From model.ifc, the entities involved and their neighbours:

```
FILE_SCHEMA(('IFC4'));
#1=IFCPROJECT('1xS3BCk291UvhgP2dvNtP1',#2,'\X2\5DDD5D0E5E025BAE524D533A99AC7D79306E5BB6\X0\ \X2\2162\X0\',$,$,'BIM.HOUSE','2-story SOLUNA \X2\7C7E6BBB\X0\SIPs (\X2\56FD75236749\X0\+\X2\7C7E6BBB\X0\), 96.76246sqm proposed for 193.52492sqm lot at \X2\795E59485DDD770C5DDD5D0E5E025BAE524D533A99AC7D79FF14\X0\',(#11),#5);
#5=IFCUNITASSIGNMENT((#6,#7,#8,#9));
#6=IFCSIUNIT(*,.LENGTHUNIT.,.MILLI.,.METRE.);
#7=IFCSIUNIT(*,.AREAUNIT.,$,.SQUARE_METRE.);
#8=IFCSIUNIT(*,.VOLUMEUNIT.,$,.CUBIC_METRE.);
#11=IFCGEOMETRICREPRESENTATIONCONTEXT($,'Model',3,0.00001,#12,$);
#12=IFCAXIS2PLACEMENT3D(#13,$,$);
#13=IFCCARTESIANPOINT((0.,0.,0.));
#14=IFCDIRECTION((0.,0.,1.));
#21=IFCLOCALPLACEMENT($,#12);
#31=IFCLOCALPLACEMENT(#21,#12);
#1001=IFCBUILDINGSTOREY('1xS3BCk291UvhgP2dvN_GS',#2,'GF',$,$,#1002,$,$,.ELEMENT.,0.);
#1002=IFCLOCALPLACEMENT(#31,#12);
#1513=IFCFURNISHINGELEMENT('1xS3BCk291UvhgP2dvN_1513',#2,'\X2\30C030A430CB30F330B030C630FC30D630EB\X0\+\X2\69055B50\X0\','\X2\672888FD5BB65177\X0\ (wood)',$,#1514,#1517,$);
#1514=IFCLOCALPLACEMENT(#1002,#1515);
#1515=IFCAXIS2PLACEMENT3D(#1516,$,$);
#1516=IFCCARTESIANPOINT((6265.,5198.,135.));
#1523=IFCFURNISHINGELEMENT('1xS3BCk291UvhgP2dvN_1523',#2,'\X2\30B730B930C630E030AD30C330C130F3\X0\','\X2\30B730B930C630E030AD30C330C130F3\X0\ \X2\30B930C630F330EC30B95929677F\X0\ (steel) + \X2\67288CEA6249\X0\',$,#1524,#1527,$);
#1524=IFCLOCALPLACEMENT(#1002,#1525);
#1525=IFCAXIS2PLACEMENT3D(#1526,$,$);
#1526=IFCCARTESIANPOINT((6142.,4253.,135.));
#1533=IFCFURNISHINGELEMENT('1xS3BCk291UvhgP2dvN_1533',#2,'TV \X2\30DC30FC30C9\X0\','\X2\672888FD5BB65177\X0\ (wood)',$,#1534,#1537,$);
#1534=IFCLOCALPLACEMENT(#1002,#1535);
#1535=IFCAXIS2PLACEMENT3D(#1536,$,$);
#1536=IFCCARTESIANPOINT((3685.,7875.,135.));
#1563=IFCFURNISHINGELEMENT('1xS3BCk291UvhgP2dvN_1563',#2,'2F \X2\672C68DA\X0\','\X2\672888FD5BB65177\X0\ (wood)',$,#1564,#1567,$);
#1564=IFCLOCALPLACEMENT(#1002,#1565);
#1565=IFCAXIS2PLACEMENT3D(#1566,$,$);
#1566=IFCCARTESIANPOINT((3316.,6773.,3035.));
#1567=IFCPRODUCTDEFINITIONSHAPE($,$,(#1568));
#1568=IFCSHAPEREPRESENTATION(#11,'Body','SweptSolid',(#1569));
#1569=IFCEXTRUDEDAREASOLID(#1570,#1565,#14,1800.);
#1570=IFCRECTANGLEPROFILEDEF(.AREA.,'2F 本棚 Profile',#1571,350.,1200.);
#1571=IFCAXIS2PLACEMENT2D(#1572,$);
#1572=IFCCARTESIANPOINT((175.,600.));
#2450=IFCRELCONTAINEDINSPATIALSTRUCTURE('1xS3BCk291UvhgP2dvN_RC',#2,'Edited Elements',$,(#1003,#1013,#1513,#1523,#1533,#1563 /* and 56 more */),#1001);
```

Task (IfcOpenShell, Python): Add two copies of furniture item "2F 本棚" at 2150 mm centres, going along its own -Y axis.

```python
import ifcopenshell
import ifcopenshell.api.geometry
import ifcopenshell.api.root
import ifcopenshell.util.element
import ifcopenshell.util.placement

model = ifcopenshell.open("model.ifc")


def reuse_history(source, copy):
    """copy_class also copies each property set's owner history, people and application; keep the originals."""
    for rel in copy.IsDefinedBy:
        if rel.is_a("IfcRelDefinesByProperties") and (history := rel.RelatingPropertyDefinition.OwnerHistory):
            rel.RelatingPropertyDefinition.OwnerHistory = source.OwnerHistory
            ifcopenshell.util.element.remove_deep2(model, history)


source = model.by_id(1563)
base = ifcopenshell.util.placement.get_local_placement(source.ObjectPlacement)
step = -base[:3, 1] * 2150.0

for i in range(1, 3):
    copy = ifcopenshell.api.root.copy_class(model, product=source)
    copy.Representation = ifcopenshell.util.element.copy_deep(
        model, source.Representation, exclude=["IfcGeometricRepresentationContext", "IfcRepresentationMap"]
    )
    reuse_history(source, copy)
    matrix = base.copy()
    matrix[:3, 3] += i * step
    print("added at", matrix[:3, 3].round(3) + 0.0)
    ifcopenshell.api.geometry.edit_object_placement(model, product=copy, matrix=matrix, is_si=False)

model.write("model_updated.ifc")
```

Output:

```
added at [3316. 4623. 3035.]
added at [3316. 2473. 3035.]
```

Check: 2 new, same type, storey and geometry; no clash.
